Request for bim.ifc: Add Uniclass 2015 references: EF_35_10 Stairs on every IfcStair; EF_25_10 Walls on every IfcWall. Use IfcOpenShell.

First a look at what the model holds.

```python
import ifcopenshell

model = ifcopenshell.open("bim.ifc")
print(model.schema)
print("classifications:", [c.Name for c in model.by_type("IfcClassification")])
for ifc_class in ("IfcDoor", "IfcRoof", "IfcStair", "IfcWall", "IfcWindow"):
    print(ifc_class, len(model.by_type(ifc_class)))
```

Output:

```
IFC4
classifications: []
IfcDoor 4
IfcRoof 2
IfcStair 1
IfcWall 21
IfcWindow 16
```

```python
import ifcopenshell
import ifcopenshell.api.classification

model = ifcopenshell.open("bim.ifc")

system = ifcopenshell.api.classification.add_classification(model, classification="Uniclass 2015")

codes = {
    "IfcStair": ("EF_35_10", "Stairs"),
    "IfcWall": ("EF_25_10", "Walls"),
}
for ifc_class, (code, name) in codes.items():
    products = model.by_type(ifc_class)
    ifcopenshell.api.classification.add_reference(
        model, products=products, classification=system, identification=code, name=name
    )
    print(code, len(products))

model.write("bim_edited.ifc")
```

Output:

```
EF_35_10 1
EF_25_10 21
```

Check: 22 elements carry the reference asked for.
